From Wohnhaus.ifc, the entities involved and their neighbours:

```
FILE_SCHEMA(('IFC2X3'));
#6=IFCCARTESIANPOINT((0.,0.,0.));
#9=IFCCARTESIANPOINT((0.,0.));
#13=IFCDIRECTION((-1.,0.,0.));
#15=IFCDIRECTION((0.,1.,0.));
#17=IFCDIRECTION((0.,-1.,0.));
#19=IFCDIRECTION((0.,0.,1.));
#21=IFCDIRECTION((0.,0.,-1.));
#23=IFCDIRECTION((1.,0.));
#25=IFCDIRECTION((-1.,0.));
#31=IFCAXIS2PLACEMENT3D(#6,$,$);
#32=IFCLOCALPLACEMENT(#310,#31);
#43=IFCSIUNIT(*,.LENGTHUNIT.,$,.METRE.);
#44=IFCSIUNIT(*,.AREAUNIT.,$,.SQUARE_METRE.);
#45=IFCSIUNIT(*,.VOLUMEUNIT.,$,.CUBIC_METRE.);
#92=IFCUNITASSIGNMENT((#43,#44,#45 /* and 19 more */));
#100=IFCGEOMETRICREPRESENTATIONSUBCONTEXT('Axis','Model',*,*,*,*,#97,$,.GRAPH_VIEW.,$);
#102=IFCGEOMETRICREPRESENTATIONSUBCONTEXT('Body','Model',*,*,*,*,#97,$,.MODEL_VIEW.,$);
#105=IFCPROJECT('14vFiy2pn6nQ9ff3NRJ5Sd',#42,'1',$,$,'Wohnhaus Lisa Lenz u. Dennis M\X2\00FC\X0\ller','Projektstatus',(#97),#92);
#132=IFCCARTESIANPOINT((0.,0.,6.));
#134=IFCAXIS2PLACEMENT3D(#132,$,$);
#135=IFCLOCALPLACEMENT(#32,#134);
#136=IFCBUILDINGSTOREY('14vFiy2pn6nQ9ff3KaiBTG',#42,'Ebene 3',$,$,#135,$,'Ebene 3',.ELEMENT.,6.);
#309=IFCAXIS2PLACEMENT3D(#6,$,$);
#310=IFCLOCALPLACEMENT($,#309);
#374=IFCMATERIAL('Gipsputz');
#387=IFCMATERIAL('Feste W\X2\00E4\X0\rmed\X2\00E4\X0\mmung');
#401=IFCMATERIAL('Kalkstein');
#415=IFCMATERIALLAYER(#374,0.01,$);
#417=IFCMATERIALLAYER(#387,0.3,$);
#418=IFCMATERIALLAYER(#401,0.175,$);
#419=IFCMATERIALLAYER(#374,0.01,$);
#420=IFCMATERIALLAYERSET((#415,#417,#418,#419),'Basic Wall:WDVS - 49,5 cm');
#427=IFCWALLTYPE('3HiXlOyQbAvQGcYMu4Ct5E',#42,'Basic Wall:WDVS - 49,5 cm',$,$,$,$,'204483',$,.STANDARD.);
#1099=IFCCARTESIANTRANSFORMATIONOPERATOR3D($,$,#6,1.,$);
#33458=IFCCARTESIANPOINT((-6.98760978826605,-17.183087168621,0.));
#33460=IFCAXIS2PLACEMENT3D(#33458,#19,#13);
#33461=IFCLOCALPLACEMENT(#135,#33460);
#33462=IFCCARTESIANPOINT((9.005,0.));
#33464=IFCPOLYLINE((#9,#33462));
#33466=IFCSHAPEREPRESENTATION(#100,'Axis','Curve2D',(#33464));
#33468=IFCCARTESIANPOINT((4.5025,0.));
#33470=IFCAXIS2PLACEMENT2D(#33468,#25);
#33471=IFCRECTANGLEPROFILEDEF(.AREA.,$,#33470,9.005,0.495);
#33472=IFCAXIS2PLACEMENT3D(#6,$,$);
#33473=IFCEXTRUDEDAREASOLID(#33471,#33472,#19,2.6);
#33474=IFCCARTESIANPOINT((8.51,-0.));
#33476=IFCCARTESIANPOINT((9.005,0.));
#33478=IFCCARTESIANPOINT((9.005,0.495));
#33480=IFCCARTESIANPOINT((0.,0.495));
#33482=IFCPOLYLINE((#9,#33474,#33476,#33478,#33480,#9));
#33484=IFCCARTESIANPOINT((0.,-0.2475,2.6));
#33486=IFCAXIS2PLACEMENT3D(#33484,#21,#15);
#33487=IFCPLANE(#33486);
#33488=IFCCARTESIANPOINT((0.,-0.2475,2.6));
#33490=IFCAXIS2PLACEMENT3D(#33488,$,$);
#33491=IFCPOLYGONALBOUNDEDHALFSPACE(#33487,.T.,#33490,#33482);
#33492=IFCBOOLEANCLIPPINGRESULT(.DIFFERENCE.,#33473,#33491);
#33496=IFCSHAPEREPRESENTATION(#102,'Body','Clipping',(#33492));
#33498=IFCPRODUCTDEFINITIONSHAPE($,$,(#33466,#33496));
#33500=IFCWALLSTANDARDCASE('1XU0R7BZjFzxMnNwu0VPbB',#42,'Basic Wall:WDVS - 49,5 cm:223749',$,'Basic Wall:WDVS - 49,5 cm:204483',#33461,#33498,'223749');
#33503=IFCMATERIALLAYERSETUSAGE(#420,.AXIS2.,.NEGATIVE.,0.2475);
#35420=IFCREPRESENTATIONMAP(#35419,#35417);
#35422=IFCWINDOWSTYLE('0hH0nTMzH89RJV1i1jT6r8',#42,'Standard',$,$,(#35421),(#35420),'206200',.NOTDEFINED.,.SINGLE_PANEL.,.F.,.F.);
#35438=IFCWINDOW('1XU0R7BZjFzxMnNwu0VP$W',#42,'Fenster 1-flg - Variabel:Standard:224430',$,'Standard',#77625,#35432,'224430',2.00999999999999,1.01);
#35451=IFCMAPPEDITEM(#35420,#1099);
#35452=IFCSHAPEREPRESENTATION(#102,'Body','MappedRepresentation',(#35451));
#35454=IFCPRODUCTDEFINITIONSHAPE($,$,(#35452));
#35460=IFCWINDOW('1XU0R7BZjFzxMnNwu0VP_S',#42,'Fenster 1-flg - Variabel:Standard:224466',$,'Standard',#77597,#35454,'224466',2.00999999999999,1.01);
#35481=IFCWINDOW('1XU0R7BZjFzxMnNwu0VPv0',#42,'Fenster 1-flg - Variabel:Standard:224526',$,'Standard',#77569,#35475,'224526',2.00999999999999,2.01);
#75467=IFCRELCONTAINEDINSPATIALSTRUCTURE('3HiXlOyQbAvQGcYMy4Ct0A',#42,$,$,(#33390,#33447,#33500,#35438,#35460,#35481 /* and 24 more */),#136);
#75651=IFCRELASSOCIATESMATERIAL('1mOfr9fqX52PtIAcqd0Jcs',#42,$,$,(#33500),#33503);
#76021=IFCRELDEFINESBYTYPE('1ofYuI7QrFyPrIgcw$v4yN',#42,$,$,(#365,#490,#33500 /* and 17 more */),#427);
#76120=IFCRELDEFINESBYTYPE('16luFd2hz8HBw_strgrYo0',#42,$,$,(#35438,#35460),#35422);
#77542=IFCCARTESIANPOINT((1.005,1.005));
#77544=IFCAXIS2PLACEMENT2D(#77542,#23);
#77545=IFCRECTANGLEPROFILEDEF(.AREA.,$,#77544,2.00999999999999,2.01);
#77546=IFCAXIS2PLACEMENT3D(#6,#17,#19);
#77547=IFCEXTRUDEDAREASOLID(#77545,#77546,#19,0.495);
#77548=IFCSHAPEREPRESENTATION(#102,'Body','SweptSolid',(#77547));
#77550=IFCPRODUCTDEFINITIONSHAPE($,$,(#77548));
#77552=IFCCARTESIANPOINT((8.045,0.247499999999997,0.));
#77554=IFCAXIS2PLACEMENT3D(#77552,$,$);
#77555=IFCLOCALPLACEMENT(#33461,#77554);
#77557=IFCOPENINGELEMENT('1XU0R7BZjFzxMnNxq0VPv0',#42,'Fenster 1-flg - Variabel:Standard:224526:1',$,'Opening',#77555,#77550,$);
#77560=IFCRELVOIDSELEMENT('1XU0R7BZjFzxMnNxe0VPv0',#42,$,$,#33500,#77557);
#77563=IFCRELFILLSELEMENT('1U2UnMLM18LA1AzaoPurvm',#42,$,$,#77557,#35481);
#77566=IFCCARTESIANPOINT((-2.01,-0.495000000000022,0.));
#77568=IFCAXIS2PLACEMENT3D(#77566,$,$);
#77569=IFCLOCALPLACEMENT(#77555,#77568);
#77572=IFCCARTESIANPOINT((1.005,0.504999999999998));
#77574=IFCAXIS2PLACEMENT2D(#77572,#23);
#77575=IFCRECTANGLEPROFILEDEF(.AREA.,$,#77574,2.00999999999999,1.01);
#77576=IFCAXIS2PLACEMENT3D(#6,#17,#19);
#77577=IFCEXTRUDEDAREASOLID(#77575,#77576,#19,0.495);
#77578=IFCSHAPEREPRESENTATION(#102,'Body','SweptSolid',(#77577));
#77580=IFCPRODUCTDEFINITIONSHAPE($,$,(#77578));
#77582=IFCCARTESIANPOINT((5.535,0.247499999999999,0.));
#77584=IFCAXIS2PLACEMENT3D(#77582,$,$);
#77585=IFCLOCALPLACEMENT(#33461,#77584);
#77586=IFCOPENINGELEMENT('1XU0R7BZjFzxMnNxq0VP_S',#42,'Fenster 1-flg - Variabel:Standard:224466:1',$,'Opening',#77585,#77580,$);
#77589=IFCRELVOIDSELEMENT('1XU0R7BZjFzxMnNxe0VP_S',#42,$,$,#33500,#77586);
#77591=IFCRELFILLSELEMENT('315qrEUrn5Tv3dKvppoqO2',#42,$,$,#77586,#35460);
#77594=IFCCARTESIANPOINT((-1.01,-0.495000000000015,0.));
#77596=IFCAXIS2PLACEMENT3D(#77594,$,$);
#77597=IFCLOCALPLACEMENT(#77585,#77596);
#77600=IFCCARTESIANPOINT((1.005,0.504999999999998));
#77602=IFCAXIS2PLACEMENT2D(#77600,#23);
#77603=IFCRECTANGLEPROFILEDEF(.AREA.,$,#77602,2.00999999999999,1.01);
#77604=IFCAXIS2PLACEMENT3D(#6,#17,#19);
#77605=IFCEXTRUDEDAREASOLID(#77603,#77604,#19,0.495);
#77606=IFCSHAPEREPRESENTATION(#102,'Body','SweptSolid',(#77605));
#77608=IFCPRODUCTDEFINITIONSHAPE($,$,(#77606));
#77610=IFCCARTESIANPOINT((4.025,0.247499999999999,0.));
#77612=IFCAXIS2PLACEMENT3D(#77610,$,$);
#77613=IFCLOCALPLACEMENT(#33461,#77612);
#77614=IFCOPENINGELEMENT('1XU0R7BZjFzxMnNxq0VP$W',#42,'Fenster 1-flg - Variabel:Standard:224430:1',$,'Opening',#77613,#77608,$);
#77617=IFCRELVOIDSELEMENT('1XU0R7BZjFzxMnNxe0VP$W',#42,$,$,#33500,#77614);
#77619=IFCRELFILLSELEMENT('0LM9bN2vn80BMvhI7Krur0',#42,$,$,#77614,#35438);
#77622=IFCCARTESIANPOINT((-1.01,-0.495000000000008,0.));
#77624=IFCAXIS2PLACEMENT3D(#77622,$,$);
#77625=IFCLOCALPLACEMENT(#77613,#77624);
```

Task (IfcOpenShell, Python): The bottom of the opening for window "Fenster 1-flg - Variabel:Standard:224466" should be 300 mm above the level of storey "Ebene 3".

```python
import numpy as np
import ifcopenshell
import ifcopenshell.api.geometry
import ifcopenshell.geom
import ifcopenshell.util.element
import ifcopenshell.util.placement
import ifcopenshell.util.shape
import ifcopenshell.util.unit

model = ifcopenshell.open("Wohnhaus.ifc")
unit_scale = ifcopenshell.util.unit.calculate_unit_scale(model)

window = model.by_guid("1XU0R7BZjFzxMnNwu0VP_S")
opening = window.FillsVoids[0].RelatingOpeningElement
storey = ifcopenshell.util.element.get_container(window, ifc_class="IfcBuildingStorey")
level = ifcopenshell.util.placement.get_local_placement(storey.ObjectPlacement)[2, 3]

# The opening's origin need not be at the sill, so measure its lowest point.
shape = ifcopenshell.geom.create_shape(ifcopenshell.geom.settings(), opening)
bottom = ifcopenshell.util.shape.get_shape_bottom_elevation(shape, shape.geometry) / unit_scale
dz = level + 0.3 / unit_scale - bottom

shift = np.array([0.0, 0.0, dz])
# The window is placed relative to its opening, so it follows when the opening moves.
matrix = ifcopenshell.util.placement.get_local_placement(opening.ObjectPlacement)
matrix[:3, 3] += shift
ifcopenshell.api.geometry.edit_object_placement(
    model, product=opening, matrix=matrix, is_si=False, should_transform_children=True
)

print(f"moved by {dz * unit_scale:+.3f} m")

model.write("Wohnhaus-out.ifc")
```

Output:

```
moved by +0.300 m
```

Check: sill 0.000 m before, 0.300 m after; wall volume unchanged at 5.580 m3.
